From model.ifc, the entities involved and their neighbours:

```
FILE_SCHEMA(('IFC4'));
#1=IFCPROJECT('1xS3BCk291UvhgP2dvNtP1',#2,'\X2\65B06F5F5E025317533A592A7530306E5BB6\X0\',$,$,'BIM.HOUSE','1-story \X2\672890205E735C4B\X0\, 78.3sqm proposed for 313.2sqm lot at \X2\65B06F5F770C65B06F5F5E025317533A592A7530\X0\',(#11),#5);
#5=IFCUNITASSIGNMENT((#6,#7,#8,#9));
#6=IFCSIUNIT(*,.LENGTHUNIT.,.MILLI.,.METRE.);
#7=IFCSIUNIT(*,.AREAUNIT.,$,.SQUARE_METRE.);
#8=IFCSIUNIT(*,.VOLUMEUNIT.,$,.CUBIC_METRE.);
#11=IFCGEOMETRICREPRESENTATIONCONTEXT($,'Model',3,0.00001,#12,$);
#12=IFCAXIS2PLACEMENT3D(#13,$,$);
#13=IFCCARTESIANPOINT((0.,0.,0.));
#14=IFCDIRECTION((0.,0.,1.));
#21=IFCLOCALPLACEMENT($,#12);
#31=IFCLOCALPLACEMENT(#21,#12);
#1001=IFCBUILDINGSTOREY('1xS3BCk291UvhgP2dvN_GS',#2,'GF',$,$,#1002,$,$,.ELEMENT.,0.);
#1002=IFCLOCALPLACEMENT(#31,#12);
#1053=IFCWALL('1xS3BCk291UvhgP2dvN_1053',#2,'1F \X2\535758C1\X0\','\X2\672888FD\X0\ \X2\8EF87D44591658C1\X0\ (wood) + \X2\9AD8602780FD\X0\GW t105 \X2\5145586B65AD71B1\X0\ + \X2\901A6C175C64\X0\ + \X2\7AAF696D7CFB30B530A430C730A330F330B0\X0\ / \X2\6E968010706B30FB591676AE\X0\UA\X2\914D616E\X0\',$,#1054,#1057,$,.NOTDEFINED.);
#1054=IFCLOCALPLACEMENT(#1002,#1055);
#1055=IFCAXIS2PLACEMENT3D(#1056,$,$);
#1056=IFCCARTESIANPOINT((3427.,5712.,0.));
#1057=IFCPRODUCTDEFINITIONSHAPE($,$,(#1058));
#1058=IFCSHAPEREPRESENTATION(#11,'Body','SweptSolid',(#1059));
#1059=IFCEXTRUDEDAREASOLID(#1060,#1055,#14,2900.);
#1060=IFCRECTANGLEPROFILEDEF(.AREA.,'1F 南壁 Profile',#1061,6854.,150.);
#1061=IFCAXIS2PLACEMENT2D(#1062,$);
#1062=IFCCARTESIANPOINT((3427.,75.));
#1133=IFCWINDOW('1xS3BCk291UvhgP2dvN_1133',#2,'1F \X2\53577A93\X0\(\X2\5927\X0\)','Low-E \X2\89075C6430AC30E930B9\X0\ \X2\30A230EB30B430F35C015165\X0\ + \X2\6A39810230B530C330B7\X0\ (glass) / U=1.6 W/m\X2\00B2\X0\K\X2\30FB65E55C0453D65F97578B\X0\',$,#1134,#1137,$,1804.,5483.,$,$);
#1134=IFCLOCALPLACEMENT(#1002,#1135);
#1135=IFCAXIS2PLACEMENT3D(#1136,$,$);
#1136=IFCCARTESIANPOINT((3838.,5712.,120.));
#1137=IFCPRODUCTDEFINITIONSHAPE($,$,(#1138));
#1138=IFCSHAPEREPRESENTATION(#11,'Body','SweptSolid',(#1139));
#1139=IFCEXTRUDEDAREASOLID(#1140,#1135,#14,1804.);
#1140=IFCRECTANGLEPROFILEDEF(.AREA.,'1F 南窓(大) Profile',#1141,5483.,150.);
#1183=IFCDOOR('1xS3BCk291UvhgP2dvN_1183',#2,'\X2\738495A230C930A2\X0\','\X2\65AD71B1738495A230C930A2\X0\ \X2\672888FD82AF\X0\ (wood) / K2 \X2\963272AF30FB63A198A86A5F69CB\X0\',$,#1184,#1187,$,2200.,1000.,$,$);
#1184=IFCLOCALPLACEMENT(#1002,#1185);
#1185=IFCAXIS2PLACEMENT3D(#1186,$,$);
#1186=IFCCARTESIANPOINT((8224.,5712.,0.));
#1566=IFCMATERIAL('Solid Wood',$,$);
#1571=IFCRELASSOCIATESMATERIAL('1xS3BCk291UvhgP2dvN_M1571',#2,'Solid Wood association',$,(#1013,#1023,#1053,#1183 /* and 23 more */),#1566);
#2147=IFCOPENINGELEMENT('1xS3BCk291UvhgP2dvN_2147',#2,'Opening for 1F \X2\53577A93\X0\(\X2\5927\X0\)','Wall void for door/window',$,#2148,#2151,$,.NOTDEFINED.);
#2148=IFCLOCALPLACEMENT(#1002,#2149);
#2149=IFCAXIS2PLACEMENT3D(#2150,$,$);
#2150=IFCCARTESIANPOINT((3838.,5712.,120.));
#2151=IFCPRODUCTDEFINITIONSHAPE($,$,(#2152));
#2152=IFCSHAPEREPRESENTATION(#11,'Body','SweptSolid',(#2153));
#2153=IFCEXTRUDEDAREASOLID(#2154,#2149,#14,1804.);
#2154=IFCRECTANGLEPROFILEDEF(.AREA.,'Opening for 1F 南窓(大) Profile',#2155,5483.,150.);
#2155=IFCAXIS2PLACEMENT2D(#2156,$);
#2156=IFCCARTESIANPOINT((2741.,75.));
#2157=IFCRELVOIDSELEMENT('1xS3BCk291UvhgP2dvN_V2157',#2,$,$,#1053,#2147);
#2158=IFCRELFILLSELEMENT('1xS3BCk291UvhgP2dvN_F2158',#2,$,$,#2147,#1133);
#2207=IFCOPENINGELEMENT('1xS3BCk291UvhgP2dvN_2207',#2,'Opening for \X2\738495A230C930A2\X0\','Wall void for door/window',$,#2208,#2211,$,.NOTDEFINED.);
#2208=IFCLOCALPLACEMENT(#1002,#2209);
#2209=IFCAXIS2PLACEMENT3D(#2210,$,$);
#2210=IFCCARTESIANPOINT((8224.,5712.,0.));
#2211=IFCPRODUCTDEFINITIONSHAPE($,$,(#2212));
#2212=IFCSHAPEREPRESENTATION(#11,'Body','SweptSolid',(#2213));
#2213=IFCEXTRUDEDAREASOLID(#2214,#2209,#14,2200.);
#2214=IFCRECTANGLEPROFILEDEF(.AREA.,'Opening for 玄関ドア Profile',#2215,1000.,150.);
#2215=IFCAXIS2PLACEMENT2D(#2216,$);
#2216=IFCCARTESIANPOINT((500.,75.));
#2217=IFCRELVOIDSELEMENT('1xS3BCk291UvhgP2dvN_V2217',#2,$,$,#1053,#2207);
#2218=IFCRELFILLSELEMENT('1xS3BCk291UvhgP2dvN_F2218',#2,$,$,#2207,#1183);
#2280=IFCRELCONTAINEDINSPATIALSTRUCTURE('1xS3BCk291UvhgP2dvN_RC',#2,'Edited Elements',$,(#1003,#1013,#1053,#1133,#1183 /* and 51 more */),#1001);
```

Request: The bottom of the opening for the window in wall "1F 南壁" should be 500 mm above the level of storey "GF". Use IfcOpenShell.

```python
import numpy as np
import ifcopenshell
import ifcopenshell.api.geometry
import ifcopenshell.geom
import ifcopenshell.util.element
import ifcopenshell.util.placement
import ifcopenshell.util.shape
import ifcopenshell.util.unit

model = ifcopenshell.open("model.ifc")
unit_scale = ifcopenshell.util.unit.calculate_unit_scale(model)

window = model.by_guid("1xS3BCk291UvhgP2dvN_1133")
opening = window.FillsVoids[0].RelatingOpeningElement
storey = ifcopenshell.util.element.get_container(window, ifc_class="IfcBuildingStorey")
level = ifcopenshell.util.placement.get_local_placement(storey.ObjectPlacement)[2, 3]

# The opening's origin need not be at the sill, so measure its lowest point.
shape = ifcopenshell.geom.create_shape(ifcopenshell.geom.settings(), opening)
bottom = ifcopenshell.util.shape.get_shape_bottom_elevation(shape, shape.geometry) / unit_scale
dz = level + 500.0 - bottom

shift = np.array([0.0, 0.0, dz])
# The window is not placed relative to its opening, so move both.
for product in (opening, window):
    matrix = ifcopenshell.util.placement.get_local_placement(product.ObjectPlacement)
    matrix[:3, 3] += shift
    ifcopenshell.api.geometry.edit_object_placement(model, product=product, matrix=matrix, is_si=False)

print(f"moved by {dz * unit_scale:+.3f} m")

model.write("model_v2.ifc")
```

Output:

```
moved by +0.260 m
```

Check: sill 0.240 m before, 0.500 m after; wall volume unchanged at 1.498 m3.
